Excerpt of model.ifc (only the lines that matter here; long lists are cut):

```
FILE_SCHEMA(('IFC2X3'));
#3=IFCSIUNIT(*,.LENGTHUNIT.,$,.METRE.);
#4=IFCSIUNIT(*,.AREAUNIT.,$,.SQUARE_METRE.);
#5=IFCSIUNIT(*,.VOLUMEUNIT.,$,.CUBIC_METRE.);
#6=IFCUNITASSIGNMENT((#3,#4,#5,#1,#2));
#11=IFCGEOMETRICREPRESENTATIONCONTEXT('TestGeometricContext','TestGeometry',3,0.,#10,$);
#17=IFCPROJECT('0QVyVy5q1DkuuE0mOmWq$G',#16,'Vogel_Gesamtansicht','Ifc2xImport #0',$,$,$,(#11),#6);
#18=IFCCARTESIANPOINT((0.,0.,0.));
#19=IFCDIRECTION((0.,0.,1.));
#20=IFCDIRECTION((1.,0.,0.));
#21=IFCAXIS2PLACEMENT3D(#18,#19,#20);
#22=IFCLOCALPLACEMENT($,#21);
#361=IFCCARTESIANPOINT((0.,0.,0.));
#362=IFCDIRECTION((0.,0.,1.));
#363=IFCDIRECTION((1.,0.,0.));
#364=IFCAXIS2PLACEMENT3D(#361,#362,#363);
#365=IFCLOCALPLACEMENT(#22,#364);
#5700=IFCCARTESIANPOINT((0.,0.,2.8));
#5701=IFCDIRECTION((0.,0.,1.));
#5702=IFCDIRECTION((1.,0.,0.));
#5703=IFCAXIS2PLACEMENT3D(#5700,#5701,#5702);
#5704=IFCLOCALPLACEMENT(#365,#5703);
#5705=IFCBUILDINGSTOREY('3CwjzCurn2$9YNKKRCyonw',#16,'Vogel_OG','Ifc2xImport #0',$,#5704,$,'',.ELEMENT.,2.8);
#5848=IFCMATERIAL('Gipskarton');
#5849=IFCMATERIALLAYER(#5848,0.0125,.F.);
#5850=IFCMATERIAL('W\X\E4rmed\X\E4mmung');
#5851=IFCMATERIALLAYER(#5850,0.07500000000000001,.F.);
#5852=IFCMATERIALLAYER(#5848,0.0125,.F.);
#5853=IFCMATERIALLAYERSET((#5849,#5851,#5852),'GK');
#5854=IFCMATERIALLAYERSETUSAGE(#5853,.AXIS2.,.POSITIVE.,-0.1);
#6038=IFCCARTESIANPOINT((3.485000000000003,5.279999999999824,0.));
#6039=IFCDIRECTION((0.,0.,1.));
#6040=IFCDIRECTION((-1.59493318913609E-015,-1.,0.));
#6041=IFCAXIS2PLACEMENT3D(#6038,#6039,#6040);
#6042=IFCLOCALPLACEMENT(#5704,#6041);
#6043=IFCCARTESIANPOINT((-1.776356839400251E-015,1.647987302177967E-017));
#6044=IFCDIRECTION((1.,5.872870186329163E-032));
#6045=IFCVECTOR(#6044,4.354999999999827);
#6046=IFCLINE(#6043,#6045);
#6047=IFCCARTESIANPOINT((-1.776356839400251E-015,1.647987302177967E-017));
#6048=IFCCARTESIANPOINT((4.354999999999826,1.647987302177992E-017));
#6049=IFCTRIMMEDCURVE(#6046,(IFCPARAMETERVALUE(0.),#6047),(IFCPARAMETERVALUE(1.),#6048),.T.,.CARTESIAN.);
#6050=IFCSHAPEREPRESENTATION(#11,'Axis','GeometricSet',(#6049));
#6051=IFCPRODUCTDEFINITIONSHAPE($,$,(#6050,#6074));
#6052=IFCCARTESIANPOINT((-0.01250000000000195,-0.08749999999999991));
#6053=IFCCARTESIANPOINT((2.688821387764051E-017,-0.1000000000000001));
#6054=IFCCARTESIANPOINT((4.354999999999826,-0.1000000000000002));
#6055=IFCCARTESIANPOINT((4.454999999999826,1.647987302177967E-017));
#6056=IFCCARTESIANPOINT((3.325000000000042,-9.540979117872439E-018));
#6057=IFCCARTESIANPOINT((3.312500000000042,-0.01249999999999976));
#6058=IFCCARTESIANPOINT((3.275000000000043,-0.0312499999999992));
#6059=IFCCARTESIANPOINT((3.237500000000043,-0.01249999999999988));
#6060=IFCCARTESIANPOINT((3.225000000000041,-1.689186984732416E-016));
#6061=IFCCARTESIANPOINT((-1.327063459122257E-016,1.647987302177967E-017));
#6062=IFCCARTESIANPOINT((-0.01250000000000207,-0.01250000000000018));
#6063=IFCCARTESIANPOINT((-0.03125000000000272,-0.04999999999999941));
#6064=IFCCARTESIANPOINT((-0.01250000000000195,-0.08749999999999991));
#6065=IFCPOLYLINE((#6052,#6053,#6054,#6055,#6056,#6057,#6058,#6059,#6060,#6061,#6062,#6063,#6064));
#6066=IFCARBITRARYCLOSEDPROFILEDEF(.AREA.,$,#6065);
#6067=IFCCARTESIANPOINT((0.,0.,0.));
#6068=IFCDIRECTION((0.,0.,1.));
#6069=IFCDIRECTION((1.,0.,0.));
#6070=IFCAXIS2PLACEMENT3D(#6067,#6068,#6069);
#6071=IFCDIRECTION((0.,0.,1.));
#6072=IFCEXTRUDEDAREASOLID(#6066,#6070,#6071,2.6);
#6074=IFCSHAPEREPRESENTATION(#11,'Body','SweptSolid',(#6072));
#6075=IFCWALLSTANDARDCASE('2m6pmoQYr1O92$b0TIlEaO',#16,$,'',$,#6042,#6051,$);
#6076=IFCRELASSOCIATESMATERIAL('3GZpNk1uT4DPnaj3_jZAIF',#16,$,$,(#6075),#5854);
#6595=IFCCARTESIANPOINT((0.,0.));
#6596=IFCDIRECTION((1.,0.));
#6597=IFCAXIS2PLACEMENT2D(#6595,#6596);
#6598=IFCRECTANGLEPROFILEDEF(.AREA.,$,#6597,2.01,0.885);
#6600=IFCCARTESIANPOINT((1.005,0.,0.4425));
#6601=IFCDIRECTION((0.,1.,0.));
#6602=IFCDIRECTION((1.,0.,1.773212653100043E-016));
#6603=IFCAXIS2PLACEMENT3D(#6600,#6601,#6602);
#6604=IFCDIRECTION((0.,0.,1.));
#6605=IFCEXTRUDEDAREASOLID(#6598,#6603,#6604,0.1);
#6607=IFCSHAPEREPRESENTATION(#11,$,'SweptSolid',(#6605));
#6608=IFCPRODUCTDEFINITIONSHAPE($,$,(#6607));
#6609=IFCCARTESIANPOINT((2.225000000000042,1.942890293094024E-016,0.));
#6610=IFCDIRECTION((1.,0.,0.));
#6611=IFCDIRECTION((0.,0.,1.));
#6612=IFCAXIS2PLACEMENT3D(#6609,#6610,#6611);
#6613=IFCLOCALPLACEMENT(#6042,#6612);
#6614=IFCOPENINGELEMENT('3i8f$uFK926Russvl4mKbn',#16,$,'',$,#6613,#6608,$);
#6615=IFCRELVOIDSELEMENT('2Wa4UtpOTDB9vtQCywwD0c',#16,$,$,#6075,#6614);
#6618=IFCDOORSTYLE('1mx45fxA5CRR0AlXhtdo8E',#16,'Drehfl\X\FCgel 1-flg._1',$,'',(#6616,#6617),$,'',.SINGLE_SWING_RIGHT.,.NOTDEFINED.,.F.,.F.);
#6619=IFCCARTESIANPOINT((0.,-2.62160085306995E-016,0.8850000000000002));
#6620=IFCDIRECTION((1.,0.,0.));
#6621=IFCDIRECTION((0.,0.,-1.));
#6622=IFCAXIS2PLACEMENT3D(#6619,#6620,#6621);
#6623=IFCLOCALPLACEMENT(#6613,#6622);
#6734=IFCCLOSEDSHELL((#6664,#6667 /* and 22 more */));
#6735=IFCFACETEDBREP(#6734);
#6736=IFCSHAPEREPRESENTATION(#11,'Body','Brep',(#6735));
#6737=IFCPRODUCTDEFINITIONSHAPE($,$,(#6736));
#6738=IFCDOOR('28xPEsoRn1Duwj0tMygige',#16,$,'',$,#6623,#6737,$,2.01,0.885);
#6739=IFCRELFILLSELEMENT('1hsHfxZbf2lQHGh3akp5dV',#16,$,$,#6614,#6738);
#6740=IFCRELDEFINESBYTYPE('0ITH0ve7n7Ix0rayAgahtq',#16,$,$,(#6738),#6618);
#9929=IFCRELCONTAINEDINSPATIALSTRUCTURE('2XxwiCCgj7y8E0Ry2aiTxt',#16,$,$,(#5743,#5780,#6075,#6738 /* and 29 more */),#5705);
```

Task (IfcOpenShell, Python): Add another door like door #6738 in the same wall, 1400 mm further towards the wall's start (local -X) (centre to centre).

```python
import ifcopenshell
import ifcopenshell.api.feature
import ifcopenshell.api.geometry
import ifcopenshell.api.root
import ifcopenshell.geom
import ifcopenshell.util.element
import ifcopenshell.util.placement
import ifcopenshell.util.shape

model = ifcopenshell.open("model.ifc")
settings = ifcopenshell.geom.settings()


def volume(element):
    """Net volume in cubic metres, openings subtracted."""
    shape = ifcopenshell.geom.create_shape(settings, element)
    return ifcopenshell.util.shape.get_volume(shape.geometry)


door = model.by_guid("28xPEsoRn1Duwj0tMygige")
opening = door.FillsVoids[0].RelatingOpeningElement
wall = opening.VoidsElements[0].RelatingBuildingElement
before = volume(wall)
shift = ifcopenshell.util.placement.get_local_placement(wall.ObjectPlacement)[:3, 0] * -1.4

# copy_class copies the void relationship, type, container and properties, but no geometry.
new_opening = ifcopenshell.api.root.copy_class(model, product=opening)
new_opening.Representation = ifcopenshell.util.element.copy_deep(
    model, opening.Representation, exclude=["IfcGeometricRepresentationContext", "IfcRepresentationMap"]
)
new_door = ifcopenshell.api.root.copy_class(model, product=door)
new_door.Representation = ifcopenshell.util.element.copy_deep(
    model, door.Representation, exclude=["IfcGeometricRepresentationContext", "IfcRepresentationMap"]
)
fills = ifcopenshell.api.feature.add_filling(model, opening=new_opening, element=new_door)
fills.OwnerHistory = new_door.OwnerHistory  # required in IFC2X3

for old, new in ((opening, new_opening), (door, new_door)):
    matrix = ifcopenshell.util.placement.get_local_placement(old.ObjectPlacement)
    matrix[:3, 3] += shift
    ifcopenshell.api.geometry.edit_object_placement(model, product=new, matrix=matrix, is_si=False)

after = volume(wall)

print(f"wall volume {before:.3f} -> {after:.3f} m3")

model.write("model_v2.ifc")
```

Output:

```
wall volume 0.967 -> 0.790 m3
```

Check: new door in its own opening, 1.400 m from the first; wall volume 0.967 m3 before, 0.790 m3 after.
